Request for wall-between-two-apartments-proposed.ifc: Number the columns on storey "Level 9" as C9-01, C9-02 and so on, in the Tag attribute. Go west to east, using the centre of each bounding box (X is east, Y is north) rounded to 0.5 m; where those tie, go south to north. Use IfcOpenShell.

First a look at what the model holds.

```python
import ifcopenshell
import ifcopenshell.util.element
import ifcopenshell.util.placement

model = ifcopenshell.open("wall-between-two-apartments-proposed.ifc")
print(model.schema)
storey = next(s for s in model.by_type("IfcBuildingStorey") if s.Name == "Level 9")
columns = [e for e in ifcopenshell.util.element.get_decomposition(storey) if e.is_a("IfcColumn")]
for e in sorted(columns, key=lambda e: e.id()):
    origin = ifcopenshell.util.placement.get_local_placement(e.ObjectPlacement)[:3, 3]
    print(e.id(), e.Tag, e.Name, origin.round(2) + 0.0, sep=" | ")
```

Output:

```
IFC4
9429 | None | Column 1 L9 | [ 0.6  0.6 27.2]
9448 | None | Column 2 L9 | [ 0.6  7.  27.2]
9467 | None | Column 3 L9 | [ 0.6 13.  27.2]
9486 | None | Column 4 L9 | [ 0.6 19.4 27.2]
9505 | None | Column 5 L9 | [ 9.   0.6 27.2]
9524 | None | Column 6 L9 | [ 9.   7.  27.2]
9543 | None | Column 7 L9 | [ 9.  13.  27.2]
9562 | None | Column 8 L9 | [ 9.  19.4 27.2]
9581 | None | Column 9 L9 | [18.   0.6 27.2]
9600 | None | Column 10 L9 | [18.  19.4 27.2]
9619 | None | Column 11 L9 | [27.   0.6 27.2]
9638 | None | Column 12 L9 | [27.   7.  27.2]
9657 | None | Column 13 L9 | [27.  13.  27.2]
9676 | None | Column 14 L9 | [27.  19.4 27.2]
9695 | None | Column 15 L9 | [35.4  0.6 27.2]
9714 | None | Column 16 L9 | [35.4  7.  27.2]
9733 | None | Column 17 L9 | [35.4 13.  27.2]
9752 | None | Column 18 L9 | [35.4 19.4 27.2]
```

```python
import ifcopenshell
import ifcopenshell.geom
import ifcopenshell.util.element
import ifcopenshell.util.shape

model = ifcopenshell.open("wall-between-two-apartments-proposed.ifc")
settings = ifcopenshell.geom.settings()
settings.set("use-world-coords", True)


def centre(element):
    shape = ifcopenshell.geom.create_shape(settings, element)
    return ifcopenshell.util.shape.get_bbox_centroid(shape.geometry)


storey = next(s for s in model.by_type("IfcBuildingStorey") if s.Name == "Level 9")
columns = [e for e in ifcopenshell.util.element.get_decomposition(storey) if e.is_a("IfcColumn")]

# Insertion points can sit at a corner or the storey origin, so sort by the geometry (in metres).
centres = {e: centre(e) for e in columns}
columns.sort(key=lambda e: (round(centres[e][0] / 0.5), centres[e][1]))

for i, e in enumerate(columns, start=1):
    number = f"C9-{i:02d}"
    e.Tag = number
    print(e.id(), number)

model.write("wall-between-two-apartments-proposed-out.ifc")
```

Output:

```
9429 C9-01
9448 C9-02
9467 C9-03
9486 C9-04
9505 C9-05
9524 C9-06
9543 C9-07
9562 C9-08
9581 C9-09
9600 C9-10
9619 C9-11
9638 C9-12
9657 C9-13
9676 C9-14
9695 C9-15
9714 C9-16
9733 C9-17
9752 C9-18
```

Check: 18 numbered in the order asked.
